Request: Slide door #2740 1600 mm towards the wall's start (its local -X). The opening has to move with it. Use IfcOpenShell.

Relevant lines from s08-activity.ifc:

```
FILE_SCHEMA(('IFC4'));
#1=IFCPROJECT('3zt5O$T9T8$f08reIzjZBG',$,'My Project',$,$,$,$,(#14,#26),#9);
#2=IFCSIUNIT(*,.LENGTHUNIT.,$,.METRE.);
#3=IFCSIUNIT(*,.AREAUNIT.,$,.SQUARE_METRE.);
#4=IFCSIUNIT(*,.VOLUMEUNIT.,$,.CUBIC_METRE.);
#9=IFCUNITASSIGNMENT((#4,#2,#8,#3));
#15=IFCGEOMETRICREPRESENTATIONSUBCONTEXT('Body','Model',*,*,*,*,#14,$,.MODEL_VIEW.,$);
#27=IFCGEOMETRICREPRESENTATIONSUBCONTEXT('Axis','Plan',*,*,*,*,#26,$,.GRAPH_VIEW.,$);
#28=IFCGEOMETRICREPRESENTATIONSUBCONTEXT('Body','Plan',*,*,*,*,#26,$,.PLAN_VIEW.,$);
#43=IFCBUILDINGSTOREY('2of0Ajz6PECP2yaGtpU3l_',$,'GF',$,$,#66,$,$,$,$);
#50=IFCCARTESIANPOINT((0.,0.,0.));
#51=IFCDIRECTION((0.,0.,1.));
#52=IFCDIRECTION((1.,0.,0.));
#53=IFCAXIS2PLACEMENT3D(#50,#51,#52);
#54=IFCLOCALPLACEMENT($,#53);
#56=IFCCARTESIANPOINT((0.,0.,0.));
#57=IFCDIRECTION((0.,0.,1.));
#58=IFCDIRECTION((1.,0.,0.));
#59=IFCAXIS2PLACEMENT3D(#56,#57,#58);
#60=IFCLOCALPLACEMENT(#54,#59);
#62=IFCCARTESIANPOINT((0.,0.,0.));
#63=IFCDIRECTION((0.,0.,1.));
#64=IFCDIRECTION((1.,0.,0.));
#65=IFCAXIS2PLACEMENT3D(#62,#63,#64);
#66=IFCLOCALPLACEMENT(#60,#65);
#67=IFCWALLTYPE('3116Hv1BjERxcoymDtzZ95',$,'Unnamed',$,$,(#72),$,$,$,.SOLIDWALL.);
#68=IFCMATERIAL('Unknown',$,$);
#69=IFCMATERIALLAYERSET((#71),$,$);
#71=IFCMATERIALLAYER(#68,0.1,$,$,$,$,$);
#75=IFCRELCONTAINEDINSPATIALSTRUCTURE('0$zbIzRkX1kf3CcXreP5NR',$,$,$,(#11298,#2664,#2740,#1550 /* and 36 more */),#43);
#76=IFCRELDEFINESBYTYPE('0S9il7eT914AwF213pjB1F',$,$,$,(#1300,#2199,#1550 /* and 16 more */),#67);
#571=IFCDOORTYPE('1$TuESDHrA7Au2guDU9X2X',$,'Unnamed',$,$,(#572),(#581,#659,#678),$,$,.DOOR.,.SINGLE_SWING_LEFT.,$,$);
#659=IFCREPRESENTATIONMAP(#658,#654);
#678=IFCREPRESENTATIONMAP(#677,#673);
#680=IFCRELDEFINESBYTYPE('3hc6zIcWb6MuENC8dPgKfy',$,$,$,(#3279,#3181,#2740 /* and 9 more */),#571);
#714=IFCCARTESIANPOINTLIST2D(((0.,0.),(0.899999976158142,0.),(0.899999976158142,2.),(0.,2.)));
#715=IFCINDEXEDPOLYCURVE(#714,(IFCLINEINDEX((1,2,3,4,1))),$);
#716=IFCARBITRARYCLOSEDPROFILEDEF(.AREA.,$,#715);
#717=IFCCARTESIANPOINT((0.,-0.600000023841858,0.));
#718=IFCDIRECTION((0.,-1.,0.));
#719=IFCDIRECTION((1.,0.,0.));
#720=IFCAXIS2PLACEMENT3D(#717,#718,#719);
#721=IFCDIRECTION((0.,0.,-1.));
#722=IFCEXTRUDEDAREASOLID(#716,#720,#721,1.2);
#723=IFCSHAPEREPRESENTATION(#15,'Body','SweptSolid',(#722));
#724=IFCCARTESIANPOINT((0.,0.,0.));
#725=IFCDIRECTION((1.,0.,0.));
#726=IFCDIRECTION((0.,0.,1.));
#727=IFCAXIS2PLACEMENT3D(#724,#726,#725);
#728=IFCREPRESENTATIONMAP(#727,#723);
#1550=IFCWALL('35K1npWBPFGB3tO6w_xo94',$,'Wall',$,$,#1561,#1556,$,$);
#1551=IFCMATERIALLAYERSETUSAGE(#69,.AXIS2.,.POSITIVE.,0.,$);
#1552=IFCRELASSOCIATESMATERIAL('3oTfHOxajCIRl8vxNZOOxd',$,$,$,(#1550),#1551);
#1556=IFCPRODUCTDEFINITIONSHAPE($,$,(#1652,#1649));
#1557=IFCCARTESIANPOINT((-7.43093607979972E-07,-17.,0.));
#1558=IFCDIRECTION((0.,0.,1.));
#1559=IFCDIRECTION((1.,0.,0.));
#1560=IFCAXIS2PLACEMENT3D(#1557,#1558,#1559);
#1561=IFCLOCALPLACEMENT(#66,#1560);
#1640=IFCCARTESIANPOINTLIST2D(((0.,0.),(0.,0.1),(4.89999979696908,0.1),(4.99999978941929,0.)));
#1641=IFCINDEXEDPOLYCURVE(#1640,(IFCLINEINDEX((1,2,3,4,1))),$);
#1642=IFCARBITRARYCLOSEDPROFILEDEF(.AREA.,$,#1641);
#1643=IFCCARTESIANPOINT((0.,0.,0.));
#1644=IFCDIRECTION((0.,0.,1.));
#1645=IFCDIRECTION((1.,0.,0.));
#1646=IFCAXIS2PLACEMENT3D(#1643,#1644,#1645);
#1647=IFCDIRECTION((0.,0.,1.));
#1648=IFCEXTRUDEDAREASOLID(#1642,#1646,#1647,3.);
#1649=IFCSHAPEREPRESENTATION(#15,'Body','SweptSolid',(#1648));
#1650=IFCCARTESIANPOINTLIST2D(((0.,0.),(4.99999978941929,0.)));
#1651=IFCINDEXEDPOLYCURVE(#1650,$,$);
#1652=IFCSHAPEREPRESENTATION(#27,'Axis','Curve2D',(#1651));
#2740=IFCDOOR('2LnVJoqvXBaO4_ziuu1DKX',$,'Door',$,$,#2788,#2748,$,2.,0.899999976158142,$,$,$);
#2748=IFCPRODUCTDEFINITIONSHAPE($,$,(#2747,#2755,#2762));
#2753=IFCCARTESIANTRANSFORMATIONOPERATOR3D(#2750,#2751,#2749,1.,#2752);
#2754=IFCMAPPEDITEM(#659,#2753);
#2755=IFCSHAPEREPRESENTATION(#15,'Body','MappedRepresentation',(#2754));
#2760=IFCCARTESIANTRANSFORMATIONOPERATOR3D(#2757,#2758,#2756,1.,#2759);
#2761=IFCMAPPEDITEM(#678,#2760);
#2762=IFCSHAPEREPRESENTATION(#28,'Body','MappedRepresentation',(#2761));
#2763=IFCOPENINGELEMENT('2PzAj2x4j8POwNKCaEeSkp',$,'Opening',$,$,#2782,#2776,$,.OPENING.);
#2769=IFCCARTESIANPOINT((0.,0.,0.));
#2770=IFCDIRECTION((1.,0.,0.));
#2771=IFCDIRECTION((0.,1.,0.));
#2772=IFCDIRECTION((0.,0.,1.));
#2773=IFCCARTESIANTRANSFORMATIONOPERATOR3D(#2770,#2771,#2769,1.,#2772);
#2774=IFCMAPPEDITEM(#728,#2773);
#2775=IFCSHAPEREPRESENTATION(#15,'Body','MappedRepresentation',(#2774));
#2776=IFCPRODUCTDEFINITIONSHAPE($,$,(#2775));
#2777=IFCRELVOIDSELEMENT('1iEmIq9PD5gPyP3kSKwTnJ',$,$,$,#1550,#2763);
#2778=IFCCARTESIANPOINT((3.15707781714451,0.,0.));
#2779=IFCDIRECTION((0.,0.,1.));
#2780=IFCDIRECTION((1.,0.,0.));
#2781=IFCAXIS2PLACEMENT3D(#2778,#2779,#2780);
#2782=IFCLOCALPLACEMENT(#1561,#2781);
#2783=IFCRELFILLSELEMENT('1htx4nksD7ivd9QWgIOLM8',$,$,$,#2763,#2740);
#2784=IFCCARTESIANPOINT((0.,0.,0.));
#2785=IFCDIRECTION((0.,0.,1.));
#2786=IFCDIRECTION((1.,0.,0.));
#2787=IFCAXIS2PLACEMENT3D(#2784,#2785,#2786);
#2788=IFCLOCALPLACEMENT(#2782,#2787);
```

```python
import ifcopenshell
import ifcopenshell.api.geometry
import ifcopenshell.util.placement

model = ifcopenshell.open("s08-activity.ifc")

door = model.by_id(2740)
opening = door.FillsVoids[0].RelatingOpeningElement
wall = opening.VoidsElements[0].RelatingBuildingElement

wall_matrix = ifcopenshell.util.placement.get_local_placement(wall.ObjectPlacement)
shift = wall_matrix[:3, 0] * -1.6
before = ifcopenshell.util.placement.get_local_placement(door.ObjectPlacement)[:3, 3].copy()

# The door is placed relative to its opening, so it follows when the opening moves.
matrix = ifcopenshell.util.placement.get_local_placement(opening.ObjectPlacement)
matrix[:3, 3] += shift
ifcopenshell.api.geometry.edit_object_placement(
    model, product=opening, matrix=matrix, is_si=False, should_transform_children=True
)

after = ifcopenshell.util.placement.get_local_placement(door.ObjectPlacement)[:3, 3]
print("door moved by", (after - before).round(3) + 0.0)

model.write("s08-activity-out.ifc")
```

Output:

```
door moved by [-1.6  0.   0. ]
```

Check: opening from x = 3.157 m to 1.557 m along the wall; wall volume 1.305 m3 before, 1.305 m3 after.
